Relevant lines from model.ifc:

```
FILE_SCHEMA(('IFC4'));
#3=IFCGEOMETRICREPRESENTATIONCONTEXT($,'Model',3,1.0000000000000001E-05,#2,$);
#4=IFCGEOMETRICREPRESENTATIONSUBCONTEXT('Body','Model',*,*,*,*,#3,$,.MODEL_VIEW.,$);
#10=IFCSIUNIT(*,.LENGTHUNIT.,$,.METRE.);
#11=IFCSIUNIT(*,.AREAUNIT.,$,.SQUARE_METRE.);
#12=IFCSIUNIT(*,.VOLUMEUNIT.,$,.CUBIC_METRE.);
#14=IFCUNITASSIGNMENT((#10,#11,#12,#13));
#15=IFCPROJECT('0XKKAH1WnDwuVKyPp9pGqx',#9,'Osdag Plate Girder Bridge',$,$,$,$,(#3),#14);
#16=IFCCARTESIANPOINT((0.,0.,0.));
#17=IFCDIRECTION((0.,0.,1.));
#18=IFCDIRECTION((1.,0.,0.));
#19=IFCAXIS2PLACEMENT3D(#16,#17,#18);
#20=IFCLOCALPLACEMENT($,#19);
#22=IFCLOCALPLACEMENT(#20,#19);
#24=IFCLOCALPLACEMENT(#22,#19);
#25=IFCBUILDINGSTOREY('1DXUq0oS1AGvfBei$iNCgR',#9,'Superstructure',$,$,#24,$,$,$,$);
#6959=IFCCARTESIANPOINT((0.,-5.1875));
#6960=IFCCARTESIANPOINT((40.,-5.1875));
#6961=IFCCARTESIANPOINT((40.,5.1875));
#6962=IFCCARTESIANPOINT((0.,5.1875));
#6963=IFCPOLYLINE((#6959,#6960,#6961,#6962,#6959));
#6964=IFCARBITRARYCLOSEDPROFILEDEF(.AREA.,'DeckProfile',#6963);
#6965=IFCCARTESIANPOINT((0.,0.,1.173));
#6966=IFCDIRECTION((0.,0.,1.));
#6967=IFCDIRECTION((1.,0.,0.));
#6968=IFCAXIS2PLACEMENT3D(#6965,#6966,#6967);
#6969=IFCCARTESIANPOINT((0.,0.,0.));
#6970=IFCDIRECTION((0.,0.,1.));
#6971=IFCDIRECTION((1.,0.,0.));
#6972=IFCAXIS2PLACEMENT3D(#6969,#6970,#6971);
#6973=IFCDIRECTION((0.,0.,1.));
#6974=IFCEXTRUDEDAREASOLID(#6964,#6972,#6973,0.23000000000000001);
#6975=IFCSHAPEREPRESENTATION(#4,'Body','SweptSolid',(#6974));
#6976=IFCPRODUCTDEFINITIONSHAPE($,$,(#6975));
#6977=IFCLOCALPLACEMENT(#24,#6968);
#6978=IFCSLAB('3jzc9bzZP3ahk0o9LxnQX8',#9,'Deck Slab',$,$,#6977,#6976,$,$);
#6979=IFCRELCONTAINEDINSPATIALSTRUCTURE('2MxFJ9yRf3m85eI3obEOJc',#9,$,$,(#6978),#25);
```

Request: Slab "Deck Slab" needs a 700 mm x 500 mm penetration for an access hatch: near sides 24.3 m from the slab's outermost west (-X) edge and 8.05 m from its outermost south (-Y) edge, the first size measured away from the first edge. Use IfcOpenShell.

```python
import numpy as np
import ifcopenshell
import ifcopenshell.api.feature
import ifcopenshell.api.geometry
import ifcopenshell.api.root
import ifcopenshell.geom
import ifcopenshell.util.placement
import ifcopenshell.util.representation
import ifcopenshell.util.shape
import ifcopenshell.util.unit

model = ifcopenshell.open("model.ifc")
unit_scale = ifcopenshell.util.unit.calculate_unit_scale(model)
settings = ifcopenshell.geom.settings()


def volume(element):
    """Net volume in cubic metres, openings subtracted."""
    shape = ifcopenshell.geom.create_shape(settings, element)
    return ifcopenshell.util.shape.get_volume(shape.geometry)


slab = model.by_guid("3jzc9bzZP3ahk0o9LxnQX8")
before = volume(slab)

# Extent in the slab's own axes, in metres. The edges named are its -X and -Y sides.
slab_shape = ifcopenshell.geom.create_shape(settings, slab)
vertices = ifcopenshell.util.shape.get_vertices(slab_shape.geometry)
x_min, y_min, bottom = vertices.min(axis=0)
top = vertices[:, 2].max()

opening = ifcopenshell.api.root.create_entity(model, ifc_class="IfcOpeningElement", name="Access hatch opening", predefined_type="OPENING")
context = ifcopenshell.util.representation.get_context(model, "Model", "Body", "MODEL_VIEW")
width, depth = 0.7, 0.5
outline = [(0.0, 0.0), (width, 0.0), (width, depth), (0.0, depth), (0.0, 0.0)]
# Overshoot both faces by 50 mm so the cut is clean.
shape = ifcopenshell.api.geometry.add_slab_representation(
    model, context=context, depth=top - bottom + 0.1, polyline=outline
)
ifcopenshell.api.geometry.assign_representation(model, product=opening, representation=shape)

matrix = ifcopenshell.util.placement.get_local_placement(slab.ObjectPlacement)
matrix[:, 3] = matrix @ np.append(np.array([x_min + 24.3, y_min + 8.05, bottom - 0.05]) / unit_scale, 1.0)
ifcopenshell.api.geometry.edit_object_placement(model, product=opening, matrix=matrix, is_si=False)
ifcopenshell.api.feature.add_feature(model, feature=opening, element=slab)

after = volume(slab)

print(f"slab volume {before:.3f} -> {after:.3f} m3")

model.write("model_edited.ifc")
```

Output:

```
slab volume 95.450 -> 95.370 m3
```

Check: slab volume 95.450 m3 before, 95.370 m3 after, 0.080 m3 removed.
